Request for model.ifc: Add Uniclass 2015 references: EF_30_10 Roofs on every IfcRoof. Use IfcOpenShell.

First a look at what the model holds.

```python
import ifcopenshell

model = ifcopenshell.open("model.ifc")
print(model.schema)
print("classifications:", [c.Name for c in model.by_type("IfcClassification")])
for ifc_class in ("IfcDoor", "IfcRoof", "IfcStair", "IfcWall", "IfcWindow"):
    print(ifc_class, len(model.by_type(ifc_class)))
```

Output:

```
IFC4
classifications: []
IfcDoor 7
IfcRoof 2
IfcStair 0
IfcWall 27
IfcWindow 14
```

```python
import ifcopenshell
import ifcopenshell.api.classification

model = ifcopenshell.open("model.ifc")

system = ifcopenshell.api.classification.add_classification(model, classification="Uniclass 2015")

codes = {
    "IfcRoof": ("EF_30_10", "Roofs"),
}
for ifc_class, (code, name) in codes.items():
    products = model.by_type(ifc_class)
    ifcopenshell.api.classification.add_reference(
        model, products=products, classification=system, identification=code, name=name
    )
    print(code, len(products))

model.write("model_edited.ifc")
```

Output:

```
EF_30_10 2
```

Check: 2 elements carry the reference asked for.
